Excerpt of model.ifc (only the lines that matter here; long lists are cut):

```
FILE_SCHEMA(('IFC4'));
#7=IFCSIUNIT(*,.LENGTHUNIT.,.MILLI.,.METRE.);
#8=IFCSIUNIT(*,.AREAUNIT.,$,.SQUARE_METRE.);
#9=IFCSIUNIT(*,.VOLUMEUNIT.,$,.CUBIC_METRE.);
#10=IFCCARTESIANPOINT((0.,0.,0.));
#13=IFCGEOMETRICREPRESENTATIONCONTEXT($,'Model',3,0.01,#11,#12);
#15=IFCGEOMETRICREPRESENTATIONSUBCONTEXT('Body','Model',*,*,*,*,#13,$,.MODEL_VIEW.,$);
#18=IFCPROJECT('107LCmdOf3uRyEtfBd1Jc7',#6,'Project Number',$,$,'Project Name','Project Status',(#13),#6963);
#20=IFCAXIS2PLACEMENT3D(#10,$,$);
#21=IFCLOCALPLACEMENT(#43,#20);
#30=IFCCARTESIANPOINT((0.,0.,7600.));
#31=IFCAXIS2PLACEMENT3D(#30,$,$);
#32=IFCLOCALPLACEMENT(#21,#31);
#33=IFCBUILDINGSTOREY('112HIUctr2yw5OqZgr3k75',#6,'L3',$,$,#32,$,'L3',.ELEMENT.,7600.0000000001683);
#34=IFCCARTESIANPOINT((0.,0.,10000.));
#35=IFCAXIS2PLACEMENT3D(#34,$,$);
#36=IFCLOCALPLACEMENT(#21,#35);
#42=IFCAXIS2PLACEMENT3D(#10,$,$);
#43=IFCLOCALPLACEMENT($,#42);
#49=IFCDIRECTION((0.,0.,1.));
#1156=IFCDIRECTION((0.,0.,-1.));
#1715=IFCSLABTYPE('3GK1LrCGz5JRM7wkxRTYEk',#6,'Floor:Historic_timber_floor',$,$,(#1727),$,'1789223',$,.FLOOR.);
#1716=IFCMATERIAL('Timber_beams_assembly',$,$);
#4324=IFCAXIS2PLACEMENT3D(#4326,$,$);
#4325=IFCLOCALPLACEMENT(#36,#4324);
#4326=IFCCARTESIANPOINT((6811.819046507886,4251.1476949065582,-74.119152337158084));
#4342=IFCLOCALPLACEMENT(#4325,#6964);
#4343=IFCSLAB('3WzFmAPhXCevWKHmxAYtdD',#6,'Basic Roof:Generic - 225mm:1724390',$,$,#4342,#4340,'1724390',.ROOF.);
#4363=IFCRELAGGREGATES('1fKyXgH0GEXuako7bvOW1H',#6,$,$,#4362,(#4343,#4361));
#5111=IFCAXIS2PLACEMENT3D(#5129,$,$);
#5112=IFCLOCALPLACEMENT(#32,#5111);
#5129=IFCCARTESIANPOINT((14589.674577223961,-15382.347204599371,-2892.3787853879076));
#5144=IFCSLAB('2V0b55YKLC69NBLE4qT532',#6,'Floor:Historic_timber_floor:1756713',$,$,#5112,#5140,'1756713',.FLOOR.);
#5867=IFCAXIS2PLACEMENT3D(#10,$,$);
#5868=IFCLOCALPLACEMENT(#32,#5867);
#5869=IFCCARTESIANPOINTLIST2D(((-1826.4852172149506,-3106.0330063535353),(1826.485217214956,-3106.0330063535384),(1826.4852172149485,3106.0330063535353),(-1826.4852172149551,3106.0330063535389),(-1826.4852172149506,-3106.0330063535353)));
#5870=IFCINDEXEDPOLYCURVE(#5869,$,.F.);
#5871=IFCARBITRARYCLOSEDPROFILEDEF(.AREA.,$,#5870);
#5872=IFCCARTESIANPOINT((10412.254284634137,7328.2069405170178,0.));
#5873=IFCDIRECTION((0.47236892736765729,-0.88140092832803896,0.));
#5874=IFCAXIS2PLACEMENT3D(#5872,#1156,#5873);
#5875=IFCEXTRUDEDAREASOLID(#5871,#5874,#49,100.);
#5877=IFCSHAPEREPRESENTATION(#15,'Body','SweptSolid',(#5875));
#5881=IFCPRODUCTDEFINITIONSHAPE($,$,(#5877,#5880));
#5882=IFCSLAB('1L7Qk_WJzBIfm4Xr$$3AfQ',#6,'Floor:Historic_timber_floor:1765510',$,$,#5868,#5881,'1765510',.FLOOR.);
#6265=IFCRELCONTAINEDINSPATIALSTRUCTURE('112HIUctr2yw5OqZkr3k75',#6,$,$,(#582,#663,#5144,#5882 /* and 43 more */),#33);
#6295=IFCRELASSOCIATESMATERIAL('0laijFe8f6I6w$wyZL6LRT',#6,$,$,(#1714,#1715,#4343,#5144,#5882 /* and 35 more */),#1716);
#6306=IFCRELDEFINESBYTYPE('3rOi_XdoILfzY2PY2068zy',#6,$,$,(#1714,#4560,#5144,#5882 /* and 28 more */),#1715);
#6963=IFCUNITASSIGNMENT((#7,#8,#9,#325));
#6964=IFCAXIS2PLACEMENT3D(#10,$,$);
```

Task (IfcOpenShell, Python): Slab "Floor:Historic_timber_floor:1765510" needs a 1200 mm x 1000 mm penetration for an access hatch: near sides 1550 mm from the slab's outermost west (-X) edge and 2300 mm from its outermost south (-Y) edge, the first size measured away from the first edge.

```python
import numpy as np
import ifcopenshell
import ifcopenshell.api.feature
import ifcopenshell.api.geometry
import ifcopenshell.api.root
import ifcopenshell.geom
import ifcopenshell.util.placement
import ifcopenshell.util.representation
import ifcopenshell.util.shape
import ifcopenshell.util.unit

model = ifcopenshell.open("model.ifc")
unit_scale = ifcopenshell.util.unit.calculate_unit_scale(model)
settings = ifcopenshell.geom.settings()


def volume(element):
    """Net volume in cubic metres, openings subtracted."""
    shape = ifcopenshell.geom.create_shape(settings, element)
    return ifcopenshell.util.shape.get_volume(shape.geometry)


slab = model.by_guid("1L7Qk_WJzBIfm4Xr$$3AfQ")
before = volume(slab)

# Extent in the slab's own axes, in metres. The edges named are its -X and -Y sides.
slab_shape = ifcopenshell.geom.create_shape(settings, slab)
vertices = ifcopenshell.util.shape.get_vertices(slab_shape.geometry)
x_min, y_min, bottom = vertices.min(axis=0)
top = vertices[:, 2].max()

opening = ifcopenshell.api.root.create_entity(model, ifc_class="IfcOpeningElement", name="Access hatch opening", predefined_type="OPENING")
context = ifcopenshell.util.representation.get_context(model, "Model", "Body", "MODEL_VIEW")
width, depth = 1.2, 1
outline = [(0.0, 0.0), (width, 0.0), (width, depth), (0.0, depth), (0.0, 0.0)]
# Overshoot both faces by 50 mm so the cut is clean.
shape = ifcopenshell.api.geometry.add_slab_representation(
    model, context=context, depth=top - bottom + 0.1, polyline=outline
)
ifcopenshell.api.geometry.assign_representation(model, product=opening, representation=shape)

matrix = ifcopenshell.util.placement.get_local_placement(slab.ObjectPlacement)
matrix[:, 3] = matrix @ np.append(np.array([x_min + 1.55, y_min + 2.3, bottom - 0.05]) / unit_scale, 1.0)
ifcopenshell.api.geometry.edit_object_placement(model, product=opening, matrix=matrix, is_si=False)
ifcopenshell.api.feature.add_feature(model, feature=opening, element=slab)

after = volume(slab)

print(f"slab volume {before:.3f} -> {after:.3f} m3")

model.write("model_edited.ifc")
```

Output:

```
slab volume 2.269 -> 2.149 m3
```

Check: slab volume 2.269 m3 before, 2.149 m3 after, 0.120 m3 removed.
